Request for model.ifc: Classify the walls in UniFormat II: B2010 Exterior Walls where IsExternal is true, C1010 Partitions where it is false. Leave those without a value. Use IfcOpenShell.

First a look at what the model holds.

```python
import ifcopenshell
import ifcopenshell.util.element

model = ifcopenshell.open("model.ifc")
print(model.schema)
print("classifications:", [c.Name for c in model.by_type("IfcClassification")])
values = [ifcopenshell.util.element.get_pset(e, "Pset_WallCommon", "IsExternal") for e in model.by_type("IfcWall")]
for value in (True, False, None):
    print("IsExternal", value, values.count(value))
```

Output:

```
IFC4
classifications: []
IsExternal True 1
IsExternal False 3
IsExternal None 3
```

```python
import ifcopenshell
import ifcopenshell.api.classification
import ifcopenshell.util.element

model = ifcopenshell.open("model.ifc")

system = ifcopenshell.api.classification.add_classification(model, classification="UniFormat II")

walls = model.by_type("IfcWall")
external = {e: ifcopenshell.util.element.get_pset(e, "Pset_WallCommon", "IsExternal") for e in walls}
for flag, code, name in ((True, "B2010", "Exterior Walls"), (False, "C1010", "Partitions")):
    products = [e for e in walls if external[e] is flag]
    ifcopenshell.api.classification.add_reference(
        model, products=products, classification=system, identification=code, name=name
    )
    print(code, len(products))

model.write("model_v2.ifc")
```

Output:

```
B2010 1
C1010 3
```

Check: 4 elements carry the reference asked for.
